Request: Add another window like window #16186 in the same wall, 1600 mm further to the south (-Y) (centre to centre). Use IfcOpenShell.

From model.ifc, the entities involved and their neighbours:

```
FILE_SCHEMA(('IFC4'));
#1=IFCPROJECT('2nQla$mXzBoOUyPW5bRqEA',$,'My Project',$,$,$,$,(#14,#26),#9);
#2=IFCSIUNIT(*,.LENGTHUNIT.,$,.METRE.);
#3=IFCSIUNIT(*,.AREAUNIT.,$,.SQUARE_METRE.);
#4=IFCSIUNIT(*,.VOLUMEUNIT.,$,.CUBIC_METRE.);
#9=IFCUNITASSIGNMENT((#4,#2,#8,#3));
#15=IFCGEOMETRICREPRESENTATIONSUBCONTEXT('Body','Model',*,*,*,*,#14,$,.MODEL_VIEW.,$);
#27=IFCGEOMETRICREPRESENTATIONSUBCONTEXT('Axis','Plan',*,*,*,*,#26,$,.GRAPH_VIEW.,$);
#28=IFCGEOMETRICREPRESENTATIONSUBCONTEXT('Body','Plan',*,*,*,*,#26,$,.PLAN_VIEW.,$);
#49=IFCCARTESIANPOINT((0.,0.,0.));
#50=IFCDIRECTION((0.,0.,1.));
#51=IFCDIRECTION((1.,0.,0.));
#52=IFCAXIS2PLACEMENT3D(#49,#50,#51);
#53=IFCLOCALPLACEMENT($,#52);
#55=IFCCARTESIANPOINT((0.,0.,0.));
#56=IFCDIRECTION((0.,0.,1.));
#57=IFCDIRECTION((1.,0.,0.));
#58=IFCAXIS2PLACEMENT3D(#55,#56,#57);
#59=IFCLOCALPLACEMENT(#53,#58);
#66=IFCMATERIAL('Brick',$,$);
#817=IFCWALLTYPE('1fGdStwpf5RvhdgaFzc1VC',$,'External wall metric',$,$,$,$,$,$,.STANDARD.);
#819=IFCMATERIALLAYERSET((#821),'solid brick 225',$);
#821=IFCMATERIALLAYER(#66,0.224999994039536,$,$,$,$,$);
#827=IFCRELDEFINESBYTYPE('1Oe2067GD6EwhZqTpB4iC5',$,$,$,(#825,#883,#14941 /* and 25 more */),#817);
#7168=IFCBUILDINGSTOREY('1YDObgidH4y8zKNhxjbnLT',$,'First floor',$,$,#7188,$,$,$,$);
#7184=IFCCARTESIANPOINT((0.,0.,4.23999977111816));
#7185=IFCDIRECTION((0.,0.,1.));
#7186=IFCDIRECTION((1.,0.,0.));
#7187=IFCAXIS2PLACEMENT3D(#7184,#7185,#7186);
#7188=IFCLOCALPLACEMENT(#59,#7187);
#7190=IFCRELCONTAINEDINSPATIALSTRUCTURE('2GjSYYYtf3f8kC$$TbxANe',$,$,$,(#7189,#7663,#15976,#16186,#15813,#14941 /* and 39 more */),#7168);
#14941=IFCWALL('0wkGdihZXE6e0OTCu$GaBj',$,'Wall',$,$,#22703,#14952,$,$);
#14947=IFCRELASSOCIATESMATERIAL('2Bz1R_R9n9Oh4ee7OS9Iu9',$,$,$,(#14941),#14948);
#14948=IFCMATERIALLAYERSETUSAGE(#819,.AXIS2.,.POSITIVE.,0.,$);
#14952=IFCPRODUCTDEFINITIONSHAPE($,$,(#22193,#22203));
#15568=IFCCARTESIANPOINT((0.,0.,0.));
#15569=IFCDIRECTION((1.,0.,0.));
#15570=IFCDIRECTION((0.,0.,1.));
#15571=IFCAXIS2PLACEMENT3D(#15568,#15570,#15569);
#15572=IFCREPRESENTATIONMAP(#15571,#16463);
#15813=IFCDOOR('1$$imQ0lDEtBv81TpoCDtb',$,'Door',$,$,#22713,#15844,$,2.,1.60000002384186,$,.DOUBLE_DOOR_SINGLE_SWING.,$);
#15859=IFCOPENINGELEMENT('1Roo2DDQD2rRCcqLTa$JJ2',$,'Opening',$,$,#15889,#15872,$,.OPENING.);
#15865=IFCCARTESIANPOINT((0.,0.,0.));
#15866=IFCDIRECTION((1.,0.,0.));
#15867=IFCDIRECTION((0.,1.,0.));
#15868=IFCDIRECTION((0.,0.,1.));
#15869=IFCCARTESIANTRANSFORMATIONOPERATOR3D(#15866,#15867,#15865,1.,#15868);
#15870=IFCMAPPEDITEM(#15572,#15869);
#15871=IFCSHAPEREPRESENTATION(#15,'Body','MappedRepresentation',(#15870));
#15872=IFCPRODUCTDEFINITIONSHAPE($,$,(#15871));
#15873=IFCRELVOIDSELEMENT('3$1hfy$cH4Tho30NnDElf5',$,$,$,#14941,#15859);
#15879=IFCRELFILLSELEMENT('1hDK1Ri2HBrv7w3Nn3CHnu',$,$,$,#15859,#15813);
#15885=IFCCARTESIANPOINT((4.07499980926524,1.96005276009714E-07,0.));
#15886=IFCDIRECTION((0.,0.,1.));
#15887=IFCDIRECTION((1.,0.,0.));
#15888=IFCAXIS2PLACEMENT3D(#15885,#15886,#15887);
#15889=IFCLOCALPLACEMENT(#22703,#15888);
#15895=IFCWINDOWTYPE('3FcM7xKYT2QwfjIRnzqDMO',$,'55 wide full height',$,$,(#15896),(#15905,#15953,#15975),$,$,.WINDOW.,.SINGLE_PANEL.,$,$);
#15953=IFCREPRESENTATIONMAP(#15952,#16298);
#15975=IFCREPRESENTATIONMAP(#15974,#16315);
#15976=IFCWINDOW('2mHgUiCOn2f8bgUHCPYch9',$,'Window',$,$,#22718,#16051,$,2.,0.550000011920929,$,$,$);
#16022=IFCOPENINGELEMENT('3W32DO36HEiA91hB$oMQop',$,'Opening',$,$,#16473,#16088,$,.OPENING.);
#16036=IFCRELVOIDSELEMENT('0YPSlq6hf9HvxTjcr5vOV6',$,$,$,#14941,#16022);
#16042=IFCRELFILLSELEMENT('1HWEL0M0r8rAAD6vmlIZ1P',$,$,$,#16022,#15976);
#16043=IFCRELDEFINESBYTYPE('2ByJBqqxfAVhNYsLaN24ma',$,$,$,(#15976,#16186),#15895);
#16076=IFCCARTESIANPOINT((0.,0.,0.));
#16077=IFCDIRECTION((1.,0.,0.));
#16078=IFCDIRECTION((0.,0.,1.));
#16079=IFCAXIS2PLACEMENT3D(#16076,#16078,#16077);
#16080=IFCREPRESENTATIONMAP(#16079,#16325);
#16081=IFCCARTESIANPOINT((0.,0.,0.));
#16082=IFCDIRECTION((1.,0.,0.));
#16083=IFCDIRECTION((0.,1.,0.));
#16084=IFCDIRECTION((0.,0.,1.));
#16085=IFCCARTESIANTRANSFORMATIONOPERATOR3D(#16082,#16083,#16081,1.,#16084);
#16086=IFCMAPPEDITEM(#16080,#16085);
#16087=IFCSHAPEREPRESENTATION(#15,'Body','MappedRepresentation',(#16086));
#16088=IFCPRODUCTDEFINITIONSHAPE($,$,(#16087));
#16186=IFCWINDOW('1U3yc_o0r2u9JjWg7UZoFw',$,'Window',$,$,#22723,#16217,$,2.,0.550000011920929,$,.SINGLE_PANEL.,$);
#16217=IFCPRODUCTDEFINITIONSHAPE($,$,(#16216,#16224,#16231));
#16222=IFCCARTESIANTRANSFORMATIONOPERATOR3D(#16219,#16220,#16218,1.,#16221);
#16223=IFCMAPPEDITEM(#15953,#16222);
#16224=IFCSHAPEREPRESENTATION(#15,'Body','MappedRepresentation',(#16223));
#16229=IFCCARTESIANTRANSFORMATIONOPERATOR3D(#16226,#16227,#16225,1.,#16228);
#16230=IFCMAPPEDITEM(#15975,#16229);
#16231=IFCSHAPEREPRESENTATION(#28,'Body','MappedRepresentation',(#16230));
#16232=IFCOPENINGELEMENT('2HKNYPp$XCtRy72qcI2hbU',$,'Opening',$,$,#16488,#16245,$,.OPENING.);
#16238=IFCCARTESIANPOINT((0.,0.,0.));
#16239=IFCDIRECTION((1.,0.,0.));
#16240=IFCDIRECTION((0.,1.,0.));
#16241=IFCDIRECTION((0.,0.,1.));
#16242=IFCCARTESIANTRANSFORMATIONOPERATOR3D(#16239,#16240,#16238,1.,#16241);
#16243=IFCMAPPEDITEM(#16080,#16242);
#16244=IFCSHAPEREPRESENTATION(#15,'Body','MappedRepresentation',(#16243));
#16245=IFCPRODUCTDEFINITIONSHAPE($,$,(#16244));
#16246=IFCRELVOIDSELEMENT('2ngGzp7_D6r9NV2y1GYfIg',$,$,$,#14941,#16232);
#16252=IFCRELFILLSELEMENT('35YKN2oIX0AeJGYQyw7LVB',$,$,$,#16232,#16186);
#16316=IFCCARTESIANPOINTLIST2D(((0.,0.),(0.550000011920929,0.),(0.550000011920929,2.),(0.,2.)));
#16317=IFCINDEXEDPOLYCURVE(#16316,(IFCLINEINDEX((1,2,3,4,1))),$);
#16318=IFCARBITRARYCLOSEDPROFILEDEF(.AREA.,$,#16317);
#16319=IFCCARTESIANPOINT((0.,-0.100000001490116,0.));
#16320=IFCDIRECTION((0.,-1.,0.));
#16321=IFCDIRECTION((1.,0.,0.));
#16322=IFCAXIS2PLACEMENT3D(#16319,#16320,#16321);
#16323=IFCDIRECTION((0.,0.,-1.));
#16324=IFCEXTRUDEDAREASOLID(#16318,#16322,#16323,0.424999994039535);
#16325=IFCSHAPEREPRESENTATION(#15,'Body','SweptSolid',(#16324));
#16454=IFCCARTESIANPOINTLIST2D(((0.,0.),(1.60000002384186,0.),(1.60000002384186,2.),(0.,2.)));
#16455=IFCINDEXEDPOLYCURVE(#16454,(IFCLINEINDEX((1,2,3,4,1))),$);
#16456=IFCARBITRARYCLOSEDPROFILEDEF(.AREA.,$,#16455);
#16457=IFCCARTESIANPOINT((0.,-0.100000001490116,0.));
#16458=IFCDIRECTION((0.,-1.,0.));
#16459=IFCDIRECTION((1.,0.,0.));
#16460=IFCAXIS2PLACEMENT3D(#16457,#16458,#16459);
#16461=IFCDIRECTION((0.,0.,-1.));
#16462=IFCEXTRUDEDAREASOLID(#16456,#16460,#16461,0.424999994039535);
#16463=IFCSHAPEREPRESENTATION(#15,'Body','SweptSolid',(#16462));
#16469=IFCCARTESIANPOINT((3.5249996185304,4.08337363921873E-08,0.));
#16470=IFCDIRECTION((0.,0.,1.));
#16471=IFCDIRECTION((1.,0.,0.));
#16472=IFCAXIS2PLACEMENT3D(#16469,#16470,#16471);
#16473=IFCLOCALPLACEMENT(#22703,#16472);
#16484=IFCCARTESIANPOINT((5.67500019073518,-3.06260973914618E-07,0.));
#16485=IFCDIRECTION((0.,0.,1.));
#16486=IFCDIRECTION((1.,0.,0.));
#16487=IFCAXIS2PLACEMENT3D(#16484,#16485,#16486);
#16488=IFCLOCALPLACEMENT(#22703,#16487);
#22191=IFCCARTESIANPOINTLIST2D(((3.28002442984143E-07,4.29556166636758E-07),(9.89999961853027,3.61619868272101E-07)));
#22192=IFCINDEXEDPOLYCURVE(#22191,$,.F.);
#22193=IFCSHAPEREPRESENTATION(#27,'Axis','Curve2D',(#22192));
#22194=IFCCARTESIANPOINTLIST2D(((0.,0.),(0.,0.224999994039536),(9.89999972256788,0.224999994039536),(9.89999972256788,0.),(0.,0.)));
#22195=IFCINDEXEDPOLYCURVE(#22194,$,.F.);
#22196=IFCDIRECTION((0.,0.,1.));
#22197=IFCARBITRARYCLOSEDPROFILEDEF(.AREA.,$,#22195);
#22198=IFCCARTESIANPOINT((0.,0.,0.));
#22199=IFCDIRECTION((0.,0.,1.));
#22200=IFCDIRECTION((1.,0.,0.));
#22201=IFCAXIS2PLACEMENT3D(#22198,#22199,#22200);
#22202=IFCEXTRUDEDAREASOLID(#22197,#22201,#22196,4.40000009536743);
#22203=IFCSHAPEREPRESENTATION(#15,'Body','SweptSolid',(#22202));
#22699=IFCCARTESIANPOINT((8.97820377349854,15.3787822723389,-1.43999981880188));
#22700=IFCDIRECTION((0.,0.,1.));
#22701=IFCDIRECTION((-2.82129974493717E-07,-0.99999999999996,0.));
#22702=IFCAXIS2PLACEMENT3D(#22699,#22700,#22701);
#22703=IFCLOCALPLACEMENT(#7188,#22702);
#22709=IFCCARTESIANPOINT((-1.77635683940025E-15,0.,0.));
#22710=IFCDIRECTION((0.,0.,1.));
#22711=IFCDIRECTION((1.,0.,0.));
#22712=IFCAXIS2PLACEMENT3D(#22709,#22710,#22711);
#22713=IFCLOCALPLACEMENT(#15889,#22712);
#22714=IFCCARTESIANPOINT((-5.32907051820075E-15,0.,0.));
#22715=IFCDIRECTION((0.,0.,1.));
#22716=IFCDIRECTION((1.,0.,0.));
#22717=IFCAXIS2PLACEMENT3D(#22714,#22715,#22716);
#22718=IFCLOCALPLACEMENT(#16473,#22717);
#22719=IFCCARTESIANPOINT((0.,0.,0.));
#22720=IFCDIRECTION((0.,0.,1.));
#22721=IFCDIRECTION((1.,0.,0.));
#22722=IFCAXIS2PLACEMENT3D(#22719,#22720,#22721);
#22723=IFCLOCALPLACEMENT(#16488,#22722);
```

```python
import ifcopenshell
import ifcopenshell.api.feature
import ifcopenshell.api.geometry
import ifcopenshell.api.root
import ifcopenshell.geom
import ifcopenshell.util.element
import ifcopenshell.util.placement
import ifcopenshell.util.shape
import ifcopenshell.util.unit

model = ifcopenshell.open("model.ifc")
unit_scale = ifcopenshell.util.unit.calculate_unit_scale(model)
settings = ifcopenshell.geom.settings()


def volume(element):
    """Net volume in cubic metres, openings subtracted."""
    shape = ifcopenshell.geom.create_shape(settings, element)
    return ifcopenshell.util.shape.get_volume(shape.geometry)


window = model.by_id(16186)
opening = window.FillsVoids[0].RelatingOpeningElement
wall = opening.VoidsElements[0].RelatingBuildingElement
before = volume(wall)
shift = ifcopenshell.util.placement.get_local_placement(wall.ObjectPlacement)[:3, 0] * 1.6 / unit_scale

# copy_class copies the void relationship, type, container and properties, but no geometry.
new_opening = ifcopenshell.api.root.copy_class(model, product=opening)
new_opening.Representation = ifcopenshell.util.element.copy_deep(
    model, opening.Representation, exclude=["IfcGeometricRepresentationContext", "IfcRepresentationMap"]
)
new_window = ifcopenshell.api.root.copy_class(model, product=window)
new_window.Representation = ifcopenshell.util.element.copy_deep(
    model, window.Representation, exclude=["IfcGeometricRepresentationContext", "IfcRepresentationMap"]
)
ifcopenshell.api.feature.add_filling(model, opening=new_opening, element=new_window)

for old, new in ((opening, new_opening), (window, new_window)):
    matrix = ifcopenshell.util.placement.get_local_placement(old.ObjectPlacement)
    matrix[:3, 3] += shift
    ifcopenshell.api.geometry.edit_object_placement(model, product=new, matrix=matrix, is_si=False)

after = volume(wall)

print(f"wall volume {before:.3f} -> {after:.3f} m3")

model.write("model_edited.ifc")
```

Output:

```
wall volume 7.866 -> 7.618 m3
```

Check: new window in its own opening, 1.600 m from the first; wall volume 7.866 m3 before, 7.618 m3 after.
